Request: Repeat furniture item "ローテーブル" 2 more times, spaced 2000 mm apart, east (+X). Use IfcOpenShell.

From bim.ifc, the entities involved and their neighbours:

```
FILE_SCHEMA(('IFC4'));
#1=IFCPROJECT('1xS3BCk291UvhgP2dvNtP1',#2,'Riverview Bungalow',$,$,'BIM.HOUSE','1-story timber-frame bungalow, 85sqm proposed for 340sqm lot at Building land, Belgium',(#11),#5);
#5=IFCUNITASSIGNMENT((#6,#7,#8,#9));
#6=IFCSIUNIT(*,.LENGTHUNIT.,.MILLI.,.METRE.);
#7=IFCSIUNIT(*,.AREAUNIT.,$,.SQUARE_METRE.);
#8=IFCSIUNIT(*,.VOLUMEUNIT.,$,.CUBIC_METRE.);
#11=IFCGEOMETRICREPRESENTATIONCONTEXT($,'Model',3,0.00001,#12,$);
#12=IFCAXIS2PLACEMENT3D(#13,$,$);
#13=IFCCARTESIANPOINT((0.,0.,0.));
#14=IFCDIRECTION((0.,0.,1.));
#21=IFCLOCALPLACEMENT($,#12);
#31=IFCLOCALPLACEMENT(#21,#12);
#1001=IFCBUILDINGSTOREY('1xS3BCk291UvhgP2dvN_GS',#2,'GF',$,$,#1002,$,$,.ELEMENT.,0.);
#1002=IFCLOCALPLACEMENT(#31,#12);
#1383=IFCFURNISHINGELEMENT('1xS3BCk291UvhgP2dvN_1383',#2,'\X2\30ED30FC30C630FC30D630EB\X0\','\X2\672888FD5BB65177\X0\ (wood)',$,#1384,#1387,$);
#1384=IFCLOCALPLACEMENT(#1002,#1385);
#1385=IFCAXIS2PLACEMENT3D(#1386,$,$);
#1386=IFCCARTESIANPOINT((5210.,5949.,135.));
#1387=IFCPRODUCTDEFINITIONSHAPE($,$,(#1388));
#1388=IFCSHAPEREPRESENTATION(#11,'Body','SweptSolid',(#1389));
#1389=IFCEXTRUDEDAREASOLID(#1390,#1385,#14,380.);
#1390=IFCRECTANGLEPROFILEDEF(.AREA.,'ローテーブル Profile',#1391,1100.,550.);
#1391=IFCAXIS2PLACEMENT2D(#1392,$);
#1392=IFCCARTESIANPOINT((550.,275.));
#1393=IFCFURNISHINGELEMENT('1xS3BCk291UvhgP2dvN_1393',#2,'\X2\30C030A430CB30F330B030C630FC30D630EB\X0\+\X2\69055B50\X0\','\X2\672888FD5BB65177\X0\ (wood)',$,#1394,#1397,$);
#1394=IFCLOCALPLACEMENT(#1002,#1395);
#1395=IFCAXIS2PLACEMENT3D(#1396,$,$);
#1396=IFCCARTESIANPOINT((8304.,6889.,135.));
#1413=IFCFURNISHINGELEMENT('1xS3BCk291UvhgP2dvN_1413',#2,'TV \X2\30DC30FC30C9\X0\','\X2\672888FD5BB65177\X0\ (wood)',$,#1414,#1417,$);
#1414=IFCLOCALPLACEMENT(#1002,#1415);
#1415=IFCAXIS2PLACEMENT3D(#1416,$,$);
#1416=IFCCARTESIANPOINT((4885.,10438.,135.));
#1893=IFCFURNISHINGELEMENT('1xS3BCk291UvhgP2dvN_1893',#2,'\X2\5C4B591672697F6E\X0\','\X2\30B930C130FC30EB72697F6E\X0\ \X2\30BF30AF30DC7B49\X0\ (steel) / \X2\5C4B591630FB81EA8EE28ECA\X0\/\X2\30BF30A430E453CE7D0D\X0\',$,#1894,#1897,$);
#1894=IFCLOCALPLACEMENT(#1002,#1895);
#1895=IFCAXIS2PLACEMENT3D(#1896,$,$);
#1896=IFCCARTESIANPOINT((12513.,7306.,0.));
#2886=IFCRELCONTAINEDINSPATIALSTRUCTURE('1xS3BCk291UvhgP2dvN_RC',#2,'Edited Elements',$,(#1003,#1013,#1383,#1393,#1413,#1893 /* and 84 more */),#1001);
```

```python
import numpy as np
import ifcopenshell
import ifcopenshell.api.geometry
import ifcopenshell.api.root
import ifcopenshell.util.element
import ifcopenshell.util.placement

model = ifcopenshell.open("bim.ifc")


def reuse_history(source, copy):
    """copy_class also copies each property set's owner history, people and application; keep the originals."""
    for rel in copy.IsDefinedBy:
        if rel.is_a("IfcRelDefinesByProperties") and (history := rel.RelatingPropertyDefinition.OwnerHistory):
            rel.RelatingPropertyDefinition.OwnerHistory = source.OwnerHistory
            ifcopenshell.util.element.remove_deep2(model, history)


source = model.by_guid("1xS3BCk291UvhgP2dvN_1383")
base = ifcopenshell.util.placement.get_local_placement(source.ObjectPlacement)
step = np.array([1.0, 0.0, 0.0]) * 2000.0

for i in range(1, 3):
    copy = ifcopenshell.api.root.copy_class(model, product=source)
    copy.Representation = ifcopenshell.util.element.copy_deep(
        model, source.Representation, exclude=["IfcGeometricRepresentationContext", "IfcRepresentationMap"]
    )
    reuse_history(source, copy)
    matrix = base.copy()
    matrix[:3, 3] += i * step
    print("added at", matrix[:3, 3].round(3) + 0.0)
    ifcopenshell.api.geometry.edit_object_placement(model, product=copy, matrix=matrix, is_si=False)

model.write("bim_edited.ifc")
```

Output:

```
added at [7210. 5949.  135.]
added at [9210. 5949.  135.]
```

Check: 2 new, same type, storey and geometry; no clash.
